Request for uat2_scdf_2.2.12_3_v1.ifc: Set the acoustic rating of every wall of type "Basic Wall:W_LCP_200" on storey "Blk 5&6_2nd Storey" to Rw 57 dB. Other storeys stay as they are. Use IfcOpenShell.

First a look at what the model holds.

```python
import ifcopenshell
import ifcopenshell.util.element

model = ifcopenshell.open("uat2_scdf_2.2.12_3_v1.ifc")
print(model.schema)
storey = next(s for s in model.by_type("IfcBuildingStorey") if s.Name == "Blk 5&6_2nd Storey")
walls = [e for e in ifcopenshell.util.element.get_decomposition(storey) if e.is_a("IfcWall")]
seen = {}
for e in walls:
    element_type = ifcopenshell.util.element.get_type(e)
    key = (element_type.Name if element_type != e and element_type else None, ifcopenshell.util.element.get_pset(e, "Pset_WallCommon", "AcousticRating"))
    seen[key] = seen.get(key, 0) + 1
for (name, value), count in sorted(seen.items(), key=str):
    print(count, "x", name, "|", value)
```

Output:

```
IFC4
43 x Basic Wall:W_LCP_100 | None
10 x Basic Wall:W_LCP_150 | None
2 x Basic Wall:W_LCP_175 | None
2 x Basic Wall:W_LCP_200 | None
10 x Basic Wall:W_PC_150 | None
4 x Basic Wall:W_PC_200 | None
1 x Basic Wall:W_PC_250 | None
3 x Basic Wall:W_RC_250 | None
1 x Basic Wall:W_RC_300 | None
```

```python
import ifcopenshell
import ifcopenshell.api.pset
import ifcopenshell.util.element

model = ifcopenshell.open("uat2_scdf_2.2.12_3_v1.ifc")

storey = next(s for s in model.by_type("IfcBuildingStorey") if s.Name == "Blk 5&6_2nd Storey")
walls = [e for e in ifcopenshell.util.element.get_decomposition(storey) if e.is_a("IfcWall")]

count = 0
for e in walls:
    element_type = ifcopenshell.util.element.get_type(e)
    if element_type in (None, e) or element_type.Name != "Basic Wall:W_LCP_200":
        continue
    # add_pset returns the element's existing set when there is one.
    pset = ifcopenshell.api.pset.add_pset(model, product=e, name="Pset_WallCommon")
    ifcopenshell.api.pset.edit_pset(model, pset=pset, properties={"AcousticRating": "Rw 57 dB"})
    count += 1

print(count, "walls updated")

model.write("uat2_scdf_2.2.12_3_v1_rev.ifc")
```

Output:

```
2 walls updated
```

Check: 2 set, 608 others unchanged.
